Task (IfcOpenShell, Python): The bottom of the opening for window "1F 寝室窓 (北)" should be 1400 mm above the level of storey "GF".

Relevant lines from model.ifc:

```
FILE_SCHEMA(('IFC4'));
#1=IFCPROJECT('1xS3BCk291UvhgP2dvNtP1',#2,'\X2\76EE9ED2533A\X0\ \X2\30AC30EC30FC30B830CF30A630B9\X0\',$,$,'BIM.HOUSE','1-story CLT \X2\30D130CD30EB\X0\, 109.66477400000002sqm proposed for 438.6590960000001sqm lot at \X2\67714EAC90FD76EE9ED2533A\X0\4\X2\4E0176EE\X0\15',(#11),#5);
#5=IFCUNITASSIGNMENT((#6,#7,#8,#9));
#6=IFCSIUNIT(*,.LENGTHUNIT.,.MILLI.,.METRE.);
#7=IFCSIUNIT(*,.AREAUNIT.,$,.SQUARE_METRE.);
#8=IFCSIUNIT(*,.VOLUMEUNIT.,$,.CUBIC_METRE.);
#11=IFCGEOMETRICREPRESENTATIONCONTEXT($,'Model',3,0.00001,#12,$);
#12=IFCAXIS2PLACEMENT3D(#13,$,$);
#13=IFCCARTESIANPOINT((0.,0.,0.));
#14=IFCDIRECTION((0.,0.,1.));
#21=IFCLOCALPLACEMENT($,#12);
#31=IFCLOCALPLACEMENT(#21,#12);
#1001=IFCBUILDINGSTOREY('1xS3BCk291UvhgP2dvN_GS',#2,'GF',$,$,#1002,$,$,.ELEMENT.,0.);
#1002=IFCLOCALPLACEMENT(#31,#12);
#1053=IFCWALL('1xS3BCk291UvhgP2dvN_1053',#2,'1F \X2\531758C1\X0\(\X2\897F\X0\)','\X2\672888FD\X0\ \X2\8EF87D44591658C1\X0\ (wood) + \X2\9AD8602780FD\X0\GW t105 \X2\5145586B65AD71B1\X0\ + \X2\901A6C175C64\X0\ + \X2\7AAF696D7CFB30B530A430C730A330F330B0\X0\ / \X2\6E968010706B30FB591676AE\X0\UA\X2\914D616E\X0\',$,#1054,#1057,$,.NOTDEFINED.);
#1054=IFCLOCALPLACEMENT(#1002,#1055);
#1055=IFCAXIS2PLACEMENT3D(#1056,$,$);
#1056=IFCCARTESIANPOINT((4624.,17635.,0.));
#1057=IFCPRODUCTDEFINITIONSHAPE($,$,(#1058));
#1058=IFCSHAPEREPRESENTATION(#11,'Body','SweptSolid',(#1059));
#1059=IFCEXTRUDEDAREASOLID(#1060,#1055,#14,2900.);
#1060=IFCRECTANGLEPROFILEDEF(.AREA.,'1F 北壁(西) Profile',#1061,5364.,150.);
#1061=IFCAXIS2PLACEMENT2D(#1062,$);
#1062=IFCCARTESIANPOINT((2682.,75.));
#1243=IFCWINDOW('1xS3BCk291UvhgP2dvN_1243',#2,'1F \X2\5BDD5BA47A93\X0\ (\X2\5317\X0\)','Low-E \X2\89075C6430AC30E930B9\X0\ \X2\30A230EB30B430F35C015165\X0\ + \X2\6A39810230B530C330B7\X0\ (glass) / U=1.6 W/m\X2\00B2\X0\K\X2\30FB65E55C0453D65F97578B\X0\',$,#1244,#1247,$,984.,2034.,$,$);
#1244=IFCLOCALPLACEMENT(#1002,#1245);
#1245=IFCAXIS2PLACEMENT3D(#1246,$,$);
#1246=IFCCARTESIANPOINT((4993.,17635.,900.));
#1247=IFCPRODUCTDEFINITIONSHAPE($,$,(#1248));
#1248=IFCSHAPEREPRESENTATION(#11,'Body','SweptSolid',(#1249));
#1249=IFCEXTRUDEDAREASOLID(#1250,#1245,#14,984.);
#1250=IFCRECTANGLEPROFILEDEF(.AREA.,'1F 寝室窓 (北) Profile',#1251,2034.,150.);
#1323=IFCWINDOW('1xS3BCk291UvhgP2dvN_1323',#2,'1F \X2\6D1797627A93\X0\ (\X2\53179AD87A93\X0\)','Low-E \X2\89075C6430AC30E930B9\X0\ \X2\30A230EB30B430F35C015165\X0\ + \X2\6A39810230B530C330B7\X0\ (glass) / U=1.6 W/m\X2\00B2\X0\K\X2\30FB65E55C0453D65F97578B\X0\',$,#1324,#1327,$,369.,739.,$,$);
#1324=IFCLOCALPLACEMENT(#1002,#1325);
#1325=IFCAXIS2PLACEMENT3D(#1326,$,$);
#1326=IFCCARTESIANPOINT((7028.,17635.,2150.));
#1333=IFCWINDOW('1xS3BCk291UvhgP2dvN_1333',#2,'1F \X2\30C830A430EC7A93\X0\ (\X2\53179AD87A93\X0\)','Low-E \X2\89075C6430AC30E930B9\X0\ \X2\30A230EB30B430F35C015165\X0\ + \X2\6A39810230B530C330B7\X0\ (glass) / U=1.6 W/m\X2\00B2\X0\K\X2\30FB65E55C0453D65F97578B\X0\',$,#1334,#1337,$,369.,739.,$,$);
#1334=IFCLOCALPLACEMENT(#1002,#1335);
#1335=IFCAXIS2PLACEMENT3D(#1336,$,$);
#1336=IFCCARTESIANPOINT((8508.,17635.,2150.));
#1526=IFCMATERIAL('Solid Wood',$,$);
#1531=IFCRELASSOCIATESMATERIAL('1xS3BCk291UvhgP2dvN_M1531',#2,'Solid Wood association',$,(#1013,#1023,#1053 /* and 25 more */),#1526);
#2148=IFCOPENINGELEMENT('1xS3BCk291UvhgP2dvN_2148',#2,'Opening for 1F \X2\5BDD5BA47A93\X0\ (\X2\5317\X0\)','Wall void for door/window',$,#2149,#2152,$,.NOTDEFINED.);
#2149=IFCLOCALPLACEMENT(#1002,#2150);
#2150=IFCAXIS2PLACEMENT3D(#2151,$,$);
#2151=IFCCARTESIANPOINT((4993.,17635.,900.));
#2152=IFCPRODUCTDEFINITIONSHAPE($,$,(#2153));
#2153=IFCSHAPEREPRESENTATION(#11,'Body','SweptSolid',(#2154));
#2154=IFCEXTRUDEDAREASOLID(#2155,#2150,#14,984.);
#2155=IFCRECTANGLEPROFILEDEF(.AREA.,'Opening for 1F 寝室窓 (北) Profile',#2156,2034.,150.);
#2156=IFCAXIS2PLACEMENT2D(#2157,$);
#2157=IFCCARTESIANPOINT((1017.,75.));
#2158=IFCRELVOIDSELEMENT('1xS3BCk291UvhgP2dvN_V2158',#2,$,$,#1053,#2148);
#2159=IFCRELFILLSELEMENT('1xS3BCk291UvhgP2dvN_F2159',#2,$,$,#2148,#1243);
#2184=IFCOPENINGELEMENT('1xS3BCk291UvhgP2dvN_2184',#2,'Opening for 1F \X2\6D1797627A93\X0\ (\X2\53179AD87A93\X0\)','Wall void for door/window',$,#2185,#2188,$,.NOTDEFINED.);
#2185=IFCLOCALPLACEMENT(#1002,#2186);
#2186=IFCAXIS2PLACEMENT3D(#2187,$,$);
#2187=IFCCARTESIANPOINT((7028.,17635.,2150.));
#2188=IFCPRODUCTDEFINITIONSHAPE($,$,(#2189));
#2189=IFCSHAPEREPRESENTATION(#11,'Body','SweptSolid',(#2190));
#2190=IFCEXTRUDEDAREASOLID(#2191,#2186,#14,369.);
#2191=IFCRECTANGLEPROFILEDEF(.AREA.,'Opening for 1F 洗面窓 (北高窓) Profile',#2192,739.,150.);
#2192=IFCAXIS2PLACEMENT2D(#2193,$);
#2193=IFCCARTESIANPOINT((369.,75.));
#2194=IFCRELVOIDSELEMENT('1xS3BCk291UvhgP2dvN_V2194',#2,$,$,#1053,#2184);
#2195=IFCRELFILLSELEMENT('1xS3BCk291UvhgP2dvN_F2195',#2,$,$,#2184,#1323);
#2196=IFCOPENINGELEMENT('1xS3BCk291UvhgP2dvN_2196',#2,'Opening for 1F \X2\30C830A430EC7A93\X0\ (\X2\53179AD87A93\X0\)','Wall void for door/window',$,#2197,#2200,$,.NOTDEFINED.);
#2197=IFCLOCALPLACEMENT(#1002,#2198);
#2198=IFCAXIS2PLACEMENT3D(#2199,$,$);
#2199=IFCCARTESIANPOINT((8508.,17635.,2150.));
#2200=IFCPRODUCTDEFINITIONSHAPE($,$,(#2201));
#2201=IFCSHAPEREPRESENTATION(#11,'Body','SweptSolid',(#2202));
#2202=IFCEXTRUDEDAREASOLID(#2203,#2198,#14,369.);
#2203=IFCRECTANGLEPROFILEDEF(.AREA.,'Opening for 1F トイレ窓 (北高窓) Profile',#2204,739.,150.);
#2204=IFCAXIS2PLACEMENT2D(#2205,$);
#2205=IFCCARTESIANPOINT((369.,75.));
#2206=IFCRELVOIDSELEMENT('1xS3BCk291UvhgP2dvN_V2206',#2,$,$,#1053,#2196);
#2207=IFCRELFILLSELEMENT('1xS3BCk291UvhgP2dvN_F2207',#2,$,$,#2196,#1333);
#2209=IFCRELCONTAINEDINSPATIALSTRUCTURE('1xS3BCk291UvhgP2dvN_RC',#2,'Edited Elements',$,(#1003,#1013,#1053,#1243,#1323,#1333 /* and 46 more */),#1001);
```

```python
import numpy as np
import ifcopenshell
import ifcopenshell.api.geometry
import ifcopenshell.geom
import ifcopenshell.util.element
import ifcopenshell.util.placement
import ifcopenshell.util.shape
import ifcopenshell.util.unit

model = ifcopenshell.open("model.ifc")
unit_scale = ifcopenshell.util.unit.calculate_unit_scale(model)

window = model.by_guid("1xS3BCk291UvhgP2dvN_1243")
opening = window.FillsVoids[0].RelatingOpeningElement
storey = ifcopenshell.util.element.get_container(window, ifc_class="IfcBuildingStorey")
level = ifcopenshell.util.placement.get_local_placement(storey.ObjectPlacement)[2, 3]

# The opening's origin need not be at the sill, so measure its lowest point.
shape = ifcopenshell.geom.create_shape(ifcopenshell.geom.settings(), opening)
bottom = ifcopenshell.util.shape.get_shape_bottom_elevation(shape, shape.geometry) / unit_scale
dz = level + 1.4 / unit_scale - bottom

shift = np.array([0.0, 0.0, dz])
# The window is not placed relative to its opening, so move both.
for product in (opening, window):
    matrix = ifcopenshell.util.placement.get_local_placement(product.ObjectPlacement)
    matrix[:3, 3] += shift
    ifcopenshell.api.geometry.edit_object_placement(model, product=product, matrix=matrix, is_si=False)

print(f"moved by {dz * unit_scale:+.3f} m")

model.write("model_edited.ifc")
```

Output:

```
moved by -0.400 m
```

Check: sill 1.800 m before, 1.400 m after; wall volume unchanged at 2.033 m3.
